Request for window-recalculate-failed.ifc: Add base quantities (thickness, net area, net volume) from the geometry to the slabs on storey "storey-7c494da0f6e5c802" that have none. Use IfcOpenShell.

First a look at what the model holds.

```python
import ifcopenshell
import ifcopenshell.util.element
import ifcopenshell.util.unit

model = ifcopenshell.open("window-recalculate-failed.ifc")
print(model.schema)
for unit_type in ("LENGTHUNIT", "AREAUNIT", "VOLUMEUNIT"):
    print(unit_type, ifcopenshell.util.unit.calculate_unit_scale(model, unit_type))
storey = next(s for s in model.by_type("IfcBuildingStorey") if s.Name == "storey-7c494da0f6e5c802")
slabs = [e for e in ifcopenshell.util.element.get_decomposition(storey) if e.is_a("IfcSlab")]
for e in sorted(slabs, key=lambda e: e.id()):
    print(e.id(), e.is_a(), e.Name, list(ifcopenshell.util.element.get_psets(e, qtos_only=True)), sep=" | ")
```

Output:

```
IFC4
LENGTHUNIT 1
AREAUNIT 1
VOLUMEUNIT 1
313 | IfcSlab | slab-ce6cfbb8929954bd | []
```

```python
import ifcopenshell
import ifcopenshell.api.pset
import ifcopenshell.geom
import ifcopenshell.util.element
import ifcopenshell.util.shape
import ifcopenshell.util.unit

model = ifcopenshell.open("window-recalculate-failed.ifc")
unit_scale = ifcopenshell.util.unit.calculate_unit_scale(model)
area_scale = ifcopenshell.util.unit.calculate_unit_scale(model, "AREAUNIT")
volume_scale = ifcopenshell.util.unit.calculate_unit_scale(model, "VOLUMEUNIT")
settings = ifcopenshell.geom.settings()

storey = next(s for s in model.by_type("IfcBuildingStorey") if s.Name == "storey-7c494da0f6e5c802")
slabs = [e for e in ifcopenshell.util.element.get_decomposition(storey) if e.is_a("IfcSlab")]

for e in sorted(slabs, key=lambda e: e.id()):
    if ifcopenshell.util.element.get_psets(e, qtos_only=True, should_inherit=False):
        continue
    # Geometry comes back in metres, in the element's own axes.
    shape = ifcopenshell.geom.create_shape(settings, e)
    values = {
        "Width": ifcopenshell.util.shape.get_z(shape.geometry) / unit_scale,
        "NetArea": ifcopenshell.util.shape.get_footprint_area(shape.geometry) / area_scale,
        "NetVolume": ifcopenshell.util.shape.get_volume(shape.geometry) / volume_scale,
    }
    qto = ifcopenshell.api.pset.add_qto(model, product=e, name="Qto_SlabBaseQuantities")
    ifcopenshell.api.pset.edit_qto(model, qto=qto, properties=values)
    print(e.id(), {k: round(v, 3) for k, v in values.items()})

model.write("window-recalculate-failed_updated.ifc")
```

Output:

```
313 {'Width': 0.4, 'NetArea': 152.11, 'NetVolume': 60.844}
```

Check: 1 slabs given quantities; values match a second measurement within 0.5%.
